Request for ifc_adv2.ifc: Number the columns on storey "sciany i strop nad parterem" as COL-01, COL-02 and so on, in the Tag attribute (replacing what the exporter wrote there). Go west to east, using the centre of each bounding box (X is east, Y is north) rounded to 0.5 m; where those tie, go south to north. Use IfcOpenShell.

First a look at what the model holds.

```python
import ifcopenshell
import ifcopenshell.util.element
import ifcopenshell.util.placement

model = ifcopenshell.open("ifc_adv2.ifc")
print(model.schema)
storey = next(s for s in model.by_type("IfcBuildingStorey") if s.Name == "sciany i strop nad parterem")
columns = [e for e in ifcopenshell.util.element.get_decomposition(storey) if e.is_a("IfcColumn")]
for e in sorted(columns, key=lambda e: e.id()):
    origin = ifcopenshell.util.placement.get_local_placement(e.ObjectPlacement)[:3, 3]
    print(e.id(), e.Tag, e.Name, origin.round(2) + 0.0, sep=" | ")
```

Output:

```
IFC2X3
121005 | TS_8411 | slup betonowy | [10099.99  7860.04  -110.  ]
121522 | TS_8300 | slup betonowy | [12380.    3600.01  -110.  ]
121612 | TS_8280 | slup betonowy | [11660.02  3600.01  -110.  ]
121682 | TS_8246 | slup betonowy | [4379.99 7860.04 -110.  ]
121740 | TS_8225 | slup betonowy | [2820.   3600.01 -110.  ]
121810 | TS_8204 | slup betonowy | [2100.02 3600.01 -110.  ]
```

```python
import ifcopenshell
import ifcopenshell.geom
import ifcopenshell.util.element
import ifcopenshell.util.shape

model = ifcopenshell.open("ifc_adv2.ifc")
settings = ifcopenshell.geom.settings()
settings.set("use-world-coords", True)


def centre(element):
    shape = ifcopenshell.geom.create_shape(settings, element)
    return ifcopenshell.util.shape.get_bbox_centroid(shape.geometry)


storey = next(s for s in model.by_type("IfcBuildingStorey") if s.Name == "sciany i strop nad parterem")
columns = [e for e in ifcopenshell.util.element.get_decomposition(storey) if e.is_a("IfcColumn")]

# Insertion points can sit at a corner or the storey origin, so sort by the geometry (in metres).
centres = {e: centre(e) for e in columns}
columns.sort(key=lambda e: (round(centres[e][0] / 0.5), centres[e][1]))

for i, e in enumerate(columns, start=1):
    number = f"COL-{i:02d}"
    e.Tag = number
    print(e.id(), number)

model.write("ifc_adv2_v2.ifc")
```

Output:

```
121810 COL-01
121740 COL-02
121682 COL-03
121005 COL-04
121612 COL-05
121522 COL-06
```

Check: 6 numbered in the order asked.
